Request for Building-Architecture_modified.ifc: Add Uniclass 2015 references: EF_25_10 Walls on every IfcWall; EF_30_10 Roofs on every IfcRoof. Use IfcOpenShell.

First a look at what the model holds.

```python
import ifcopenshell

model = ifcopenshell.open("Building-Architecture_modified.ifc")
print(model.schema)
print("classifications:", [c.Name for c in model.by_type("IfcClassification")])
for ifc_class in ("IfcDoor", "IfcRoof", "IfcStair", "IfcWall", "IfcWindow"):
    print(ifc_class, len(model.by_type(ifc_class)))
```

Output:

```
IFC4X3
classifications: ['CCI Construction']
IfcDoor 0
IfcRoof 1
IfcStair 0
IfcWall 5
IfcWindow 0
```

```python
import ifcopenshell
import ifcopenshell.api.classification

model = ifcopenshell.open("Building-Architecture_modified.ifc")

system = ifcopenshell.api.classification.add_classification(model, classification="Uniclass 2015")

codes = {
    "IfcWall": ("EF_25_10", "Walls"),
    "IfcRoof": ("EF_30_10", "Roofs"),
}
for ifc_class, (code, name) in codes.items():
    products = model.by_type(ifc_class)
    ifcopenshell.api.classification.add_reference(
        model, products=products, classification=system, identification=code, name=name
    )
    print(code, len(products))

model.write("Building-Architecture_modified-out.ifc")
```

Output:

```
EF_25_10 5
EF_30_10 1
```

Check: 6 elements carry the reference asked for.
